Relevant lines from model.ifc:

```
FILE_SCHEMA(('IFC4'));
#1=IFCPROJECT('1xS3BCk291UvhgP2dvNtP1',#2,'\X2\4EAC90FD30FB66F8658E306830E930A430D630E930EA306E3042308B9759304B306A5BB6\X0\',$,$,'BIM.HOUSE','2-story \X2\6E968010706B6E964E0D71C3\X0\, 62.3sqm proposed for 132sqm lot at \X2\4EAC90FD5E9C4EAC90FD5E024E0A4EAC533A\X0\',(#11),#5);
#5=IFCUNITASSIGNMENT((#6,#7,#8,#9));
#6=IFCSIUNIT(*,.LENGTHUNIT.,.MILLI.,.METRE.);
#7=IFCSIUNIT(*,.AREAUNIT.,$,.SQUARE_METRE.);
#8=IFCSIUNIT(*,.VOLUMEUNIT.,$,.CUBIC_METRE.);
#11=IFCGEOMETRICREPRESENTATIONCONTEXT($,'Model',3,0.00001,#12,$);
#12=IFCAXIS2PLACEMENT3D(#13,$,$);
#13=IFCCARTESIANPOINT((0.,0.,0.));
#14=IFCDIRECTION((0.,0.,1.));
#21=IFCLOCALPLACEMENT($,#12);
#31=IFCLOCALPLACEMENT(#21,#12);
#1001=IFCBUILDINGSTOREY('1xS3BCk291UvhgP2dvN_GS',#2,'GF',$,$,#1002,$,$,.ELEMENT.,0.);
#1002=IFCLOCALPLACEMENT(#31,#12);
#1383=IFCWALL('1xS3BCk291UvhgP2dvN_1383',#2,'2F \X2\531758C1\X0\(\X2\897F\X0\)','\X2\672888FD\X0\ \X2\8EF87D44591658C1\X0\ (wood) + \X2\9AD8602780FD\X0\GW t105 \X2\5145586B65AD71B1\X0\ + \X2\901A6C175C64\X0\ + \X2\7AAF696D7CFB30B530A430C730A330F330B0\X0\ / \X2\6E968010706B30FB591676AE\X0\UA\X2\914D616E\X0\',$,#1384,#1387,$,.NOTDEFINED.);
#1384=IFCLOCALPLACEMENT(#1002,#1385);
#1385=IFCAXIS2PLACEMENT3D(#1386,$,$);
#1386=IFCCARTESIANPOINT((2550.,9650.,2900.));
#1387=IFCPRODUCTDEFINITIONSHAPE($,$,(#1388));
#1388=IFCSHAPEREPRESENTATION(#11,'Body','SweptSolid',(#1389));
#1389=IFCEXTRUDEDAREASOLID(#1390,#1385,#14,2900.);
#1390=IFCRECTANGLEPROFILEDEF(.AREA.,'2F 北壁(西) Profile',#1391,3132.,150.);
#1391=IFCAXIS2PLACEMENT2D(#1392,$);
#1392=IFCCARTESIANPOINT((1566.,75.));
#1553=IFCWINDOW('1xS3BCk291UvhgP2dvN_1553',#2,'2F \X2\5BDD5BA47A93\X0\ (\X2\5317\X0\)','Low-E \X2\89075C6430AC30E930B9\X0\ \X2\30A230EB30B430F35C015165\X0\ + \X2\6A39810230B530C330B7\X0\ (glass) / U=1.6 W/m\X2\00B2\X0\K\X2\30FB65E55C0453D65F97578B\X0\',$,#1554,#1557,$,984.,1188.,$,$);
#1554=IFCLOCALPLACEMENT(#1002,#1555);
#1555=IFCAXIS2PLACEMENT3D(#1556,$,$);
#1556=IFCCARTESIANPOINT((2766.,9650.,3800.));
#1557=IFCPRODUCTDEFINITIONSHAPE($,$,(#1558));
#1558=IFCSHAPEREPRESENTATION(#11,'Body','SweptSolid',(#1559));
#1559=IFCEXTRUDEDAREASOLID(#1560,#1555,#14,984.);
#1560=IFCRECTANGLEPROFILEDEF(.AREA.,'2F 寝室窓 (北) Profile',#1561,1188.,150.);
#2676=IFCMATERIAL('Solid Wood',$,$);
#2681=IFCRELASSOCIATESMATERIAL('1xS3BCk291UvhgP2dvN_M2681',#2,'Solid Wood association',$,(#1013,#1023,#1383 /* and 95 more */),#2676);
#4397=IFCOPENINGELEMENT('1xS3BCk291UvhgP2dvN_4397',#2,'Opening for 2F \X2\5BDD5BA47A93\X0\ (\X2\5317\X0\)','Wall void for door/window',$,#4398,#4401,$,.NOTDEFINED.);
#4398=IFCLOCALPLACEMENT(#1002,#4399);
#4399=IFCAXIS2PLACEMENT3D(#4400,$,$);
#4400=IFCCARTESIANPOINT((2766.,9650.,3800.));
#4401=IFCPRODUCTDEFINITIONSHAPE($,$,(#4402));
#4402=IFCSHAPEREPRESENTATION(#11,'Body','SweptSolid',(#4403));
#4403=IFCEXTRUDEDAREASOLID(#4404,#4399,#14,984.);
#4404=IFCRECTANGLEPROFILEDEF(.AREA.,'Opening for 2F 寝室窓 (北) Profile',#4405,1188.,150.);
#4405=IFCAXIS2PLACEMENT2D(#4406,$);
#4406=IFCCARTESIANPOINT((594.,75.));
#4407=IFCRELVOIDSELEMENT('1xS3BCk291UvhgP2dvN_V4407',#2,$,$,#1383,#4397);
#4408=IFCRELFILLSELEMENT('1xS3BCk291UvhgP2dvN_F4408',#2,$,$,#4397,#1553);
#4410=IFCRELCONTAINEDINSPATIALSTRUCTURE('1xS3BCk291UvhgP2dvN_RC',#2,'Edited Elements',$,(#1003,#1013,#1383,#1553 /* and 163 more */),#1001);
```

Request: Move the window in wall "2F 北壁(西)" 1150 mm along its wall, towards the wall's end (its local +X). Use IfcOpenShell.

```python
import ifcopenshell
import ifcopenshell.api.geometry
import ifcopenshell.util.placement

model = ifcopenshell.open("model.ifc")

window = model.by_guid("1xS3BCk291UvhgP2dvN_1553")
opening = window.FillsVoids[0].RelatingOpeningElement
wall = opening.VoidsElements[0].RelatingBuildingElement

wall_matrix = ifcopenshell.util.placement.get_local_placement(wall.ObjectPlacement)
shift = wall_matrix[:3, 0] * 1150.0
before = ifcopenshell.util.placement.get_local_placement(window.ObjectPlacement)[:3, 3].copy()

# The window is not placed relative to its opening, so move both.
for product in (opening, window):
    matrix = ifcopenshell.util.placement.get_local_placement(product.ObjectPlacement)
    matrix[:3, 3] += shift
    ifcopenshell.api.geometry.edit_object_placement(model, product=product, matrix=matrix, is_si=False)

after = ifcopenshell.util.placement.get_local_placement(window.ObjectPlacement)[:3, 3]
print("window moved by", (after - before).round(3) + 0.0)

model.write("model_updated.ifc")
```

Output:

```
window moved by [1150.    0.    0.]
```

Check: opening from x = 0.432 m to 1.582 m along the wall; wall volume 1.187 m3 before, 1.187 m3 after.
